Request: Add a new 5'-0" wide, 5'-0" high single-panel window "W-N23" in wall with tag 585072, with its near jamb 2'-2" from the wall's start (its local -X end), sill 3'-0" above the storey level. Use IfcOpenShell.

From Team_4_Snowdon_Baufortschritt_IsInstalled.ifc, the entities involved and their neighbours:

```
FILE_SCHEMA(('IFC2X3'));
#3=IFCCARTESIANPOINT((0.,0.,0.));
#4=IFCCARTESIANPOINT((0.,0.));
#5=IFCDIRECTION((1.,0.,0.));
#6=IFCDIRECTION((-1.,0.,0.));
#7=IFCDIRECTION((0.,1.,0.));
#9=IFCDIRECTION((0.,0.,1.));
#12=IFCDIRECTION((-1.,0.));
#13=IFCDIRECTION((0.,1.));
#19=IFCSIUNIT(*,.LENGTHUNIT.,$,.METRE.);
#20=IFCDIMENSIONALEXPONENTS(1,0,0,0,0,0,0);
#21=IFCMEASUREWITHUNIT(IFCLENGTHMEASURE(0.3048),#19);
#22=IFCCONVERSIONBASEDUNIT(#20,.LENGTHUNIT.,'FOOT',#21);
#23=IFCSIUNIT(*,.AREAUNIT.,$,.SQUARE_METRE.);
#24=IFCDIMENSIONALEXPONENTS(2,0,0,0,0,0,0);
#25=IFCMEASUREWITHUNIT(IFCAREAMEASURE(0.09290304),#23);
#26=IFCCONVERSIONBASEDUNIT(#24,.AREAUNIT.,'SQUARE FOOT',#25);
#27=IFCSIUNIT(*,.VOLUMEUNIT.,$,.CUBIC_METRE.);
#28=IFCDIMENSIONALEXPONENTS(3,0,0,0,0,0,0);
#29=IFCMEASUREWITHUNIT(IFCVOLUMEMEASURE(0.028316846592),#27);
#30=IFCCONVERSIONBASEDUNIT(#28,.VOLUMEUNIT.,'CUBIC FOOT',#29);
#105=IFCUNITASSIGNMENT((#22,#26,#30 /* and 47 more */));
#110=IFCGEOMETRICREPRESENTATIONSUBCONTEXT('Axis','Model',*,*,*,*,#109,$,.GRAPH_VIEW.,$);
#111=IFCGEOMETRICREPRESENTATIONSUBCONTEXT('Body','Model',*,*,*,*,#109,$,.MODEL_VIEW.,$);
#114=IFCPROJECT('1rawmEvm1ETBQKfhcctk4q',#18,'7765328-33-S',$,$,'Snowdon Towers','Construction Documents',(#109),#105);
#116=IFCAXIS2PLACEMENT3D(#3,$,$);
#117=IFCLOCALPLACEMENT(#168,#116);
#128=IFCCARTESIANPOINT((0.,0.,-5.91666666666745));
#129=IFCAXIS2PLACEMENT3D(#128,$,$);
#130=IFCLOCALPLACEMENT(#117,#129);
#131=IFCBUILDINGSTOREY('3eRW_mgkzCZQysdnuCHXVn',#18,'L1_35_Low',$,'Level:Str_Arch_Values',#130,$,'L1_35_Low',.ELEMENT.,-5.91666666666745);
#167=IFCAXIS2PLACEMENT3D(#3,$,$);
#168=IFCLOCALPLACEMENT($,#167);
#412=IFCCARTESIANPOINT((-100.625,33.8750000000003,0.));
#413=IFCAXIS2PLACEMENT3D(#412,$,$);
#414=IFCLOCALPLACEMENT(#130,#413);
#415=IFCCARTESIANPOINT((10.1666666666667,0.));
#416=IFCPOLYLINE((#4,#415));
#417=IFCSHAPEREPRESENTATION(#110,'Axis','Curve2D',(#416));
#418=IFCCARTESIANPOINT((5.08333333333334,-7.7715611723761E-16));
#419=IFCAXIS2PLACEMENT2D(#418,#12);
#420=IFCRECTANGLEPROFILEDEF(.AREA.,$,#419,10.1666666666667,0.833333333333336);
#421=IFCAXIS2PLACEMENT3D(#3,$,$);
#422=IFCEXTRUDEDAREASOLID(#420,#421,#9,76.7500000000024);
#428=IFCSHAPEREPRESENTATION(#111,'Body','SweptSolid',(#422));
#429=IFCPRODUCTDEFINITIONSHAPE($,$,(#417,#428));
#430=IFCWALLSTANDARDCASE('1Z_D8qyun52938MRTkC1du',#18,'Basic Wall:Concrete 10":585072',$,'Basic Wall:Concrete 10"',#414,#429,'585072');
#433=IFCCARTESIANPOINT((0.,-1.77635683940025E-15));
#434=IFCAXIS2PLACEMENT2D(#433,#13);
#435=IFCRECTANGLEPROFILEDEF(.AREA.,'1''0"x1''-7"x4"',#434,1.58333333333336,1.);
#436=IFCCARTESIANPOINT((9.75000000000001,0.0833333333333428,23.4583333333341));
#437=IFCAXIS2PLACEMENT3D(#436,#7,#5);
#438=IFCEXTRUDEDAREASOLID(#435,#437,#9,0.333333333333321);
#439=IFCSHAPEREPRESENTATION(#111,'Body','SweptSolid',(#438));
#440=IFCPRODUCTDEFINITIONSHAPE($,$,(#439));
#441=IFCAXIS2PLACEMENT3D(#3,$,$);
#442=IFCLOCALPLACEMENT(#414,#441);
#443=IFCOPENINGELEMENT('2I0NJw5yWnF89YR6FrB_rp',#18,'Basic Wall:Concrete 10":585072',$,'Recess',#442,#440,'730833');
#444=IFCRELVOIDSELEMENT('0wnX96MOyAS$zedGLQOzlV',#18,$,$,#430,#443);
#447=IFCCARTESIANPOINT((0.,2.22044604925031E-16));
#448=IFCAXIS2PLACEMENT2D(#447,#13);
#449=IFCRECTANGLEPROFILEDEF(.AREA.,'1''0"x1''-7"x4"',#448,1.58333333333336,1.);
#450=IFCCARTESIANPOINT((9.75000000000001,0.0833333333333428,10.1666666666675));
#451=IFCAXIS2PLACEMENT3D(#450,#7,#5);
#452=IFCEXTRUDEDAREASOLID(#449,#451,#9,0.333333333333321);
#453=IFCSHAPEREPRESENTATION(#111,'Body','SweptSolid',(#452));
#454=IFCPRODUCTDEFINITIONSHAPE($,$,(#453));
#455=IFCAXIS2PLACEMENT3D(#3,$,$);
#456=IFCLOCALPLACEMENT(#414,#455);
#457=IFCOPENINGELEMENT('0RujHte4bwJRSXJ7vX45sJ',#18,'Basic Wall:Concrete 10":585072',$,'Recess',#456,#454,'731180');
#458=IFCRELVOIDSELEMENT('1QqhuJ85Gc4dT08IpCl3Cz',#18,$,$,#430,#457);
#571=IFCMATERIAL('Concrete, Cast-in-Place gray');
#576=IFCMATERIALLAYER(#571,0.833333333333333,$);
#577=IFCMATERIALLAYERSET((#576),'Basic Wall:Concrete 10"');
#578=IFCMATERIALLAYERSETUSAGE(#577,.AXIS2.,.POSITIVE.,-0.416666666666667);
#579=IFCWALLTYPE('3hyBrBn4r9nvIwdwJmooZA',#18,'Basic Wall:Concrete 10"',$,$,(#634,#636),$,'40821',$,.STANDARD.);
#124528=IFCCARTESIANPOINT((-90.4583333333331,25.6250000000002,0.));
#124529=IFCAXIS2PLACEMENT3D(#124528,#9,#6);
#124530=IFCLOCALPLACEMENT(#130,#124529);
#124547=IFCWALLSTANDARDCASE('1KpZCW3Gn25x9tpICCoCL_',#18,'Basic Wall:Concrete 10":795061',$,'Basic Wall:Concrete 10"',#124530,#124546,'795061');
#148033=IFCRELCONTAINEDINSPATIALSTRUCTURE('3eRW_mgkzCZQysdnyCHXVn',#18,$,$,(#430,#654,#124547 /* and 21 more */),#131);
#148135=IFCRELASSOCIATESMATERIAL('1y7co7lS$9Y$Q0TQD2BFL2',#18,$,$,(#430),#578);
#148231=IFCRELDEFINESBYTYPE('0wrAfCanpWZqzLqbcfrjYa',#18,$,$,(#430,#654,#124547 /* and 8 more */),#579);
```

```python
import numpy as np
import ifcopenshell
import ifcopenshell.api.feature
import ifcopenshell.api.geometry
import ifcopenshell.api.root
import ifcopenshell.api.spatial
import ifcopenshell.api.type
import ifcopenshell.geom
import ifcopenshell.util.element
import ifcopenshell.util.placement
import ifcopenshell.util.representation
import ifcopenshell.util.shape
import ifcopenshell.util.unit

model = ifcopenshell.open("Team_4_Snowdon_Baufortschritt_IsInstalled.ifc")
unit_scale = ifcopenshell.util.unit.calculate_unit_scale(model)
settings = ifcopenshell.geom.settings()


def volume(element):
    """Net volume in cubic metres, openings subtracted."""
    shape = ifcopenshell.geom.create_shape(settings, element)
    return ifcopenshell.util.shape.get_volume(shape.geometry)


wall = model.by_guid("1Z_D8qyun52938MRTkC1du")
storey = ifcopenshell.util.element.get_container(wall, ifc_class="IfcBuildingStorey")
context = ifcopenshell.util.representation.get_context(model, "Model", "Body", "MODEL_VIEW")
before = volume(wall)

width, height, from_end, sill = 1.524, 1.524, 0.6604, 0.9144  # metres

# The wall runs along its own X axis, and the end named is its -X end.
wall_shape = ifcopenshell.geom.create_shape(settings, wall)
x, y, z = ifcopenshell.util.shape.get_vertices(wall_shape.geometry).T
start = x.min() + from_end
face, thickness = float(y.min()), float(y.max() - y.min())
wall_matrix = ifcopenshell.util.placement.get_local_placement(wall.ObjectPlacement)
level = ifcopenshell.util.placement.get_local_placement(storey.ObjectPlacement)[2, 3]


def in_wall(x, y):
    """Placement at x, y metres in the wall's axes, at sill height."""
    matrix = wall_matrix.copy()
    matrix[:, 3] = wall_matrix @ np.array([x / unit_scale, y / unit_scale, 0.0, 1.0])
    matrix[2, 3] = level + sill / unit_scale
    return matrix


# Opening: a box that overshoots both wall faces by 50 mm.
opening = ifcopenshell.api.root.create_entity(model, ifc_class="IfcOpeningElement")
box = ifcopenshell.api.geometry.add_wall_representation(
    model, context=context, length=width, height=height, thickness=thickness + 0.1
)
ifcopenshell.api.geometry.assign_representation(model, product=opening, representation=box)
ifcopenshell.api.geometry.edit_object_placement(model, product=opening, matrix=in_wall(start, face - 0.05), is_si=False)
ifcopenshell.api.feature.add_feature(model, feature=opening, element=wall)

window = ifcopenshell.api.root.create_entity(model, ifc_class="IfcWindow", name="W-N23")
window.OverallWidth, window.OverallHeight = width / unit_scale, height / unit_scale
body = ifcopenshell.api.geometry.add_window_representation(
    model,
    context=context,
    overall_width=window.OverallWidth,
    overall_height=window.OverallHeight,
    partition_type="SINGLE_PANEL",
)
ifcopenshell.api.geometry.assign_representation(model, product=window, representation=body)
ifcopenshell.api.spatial.assign_container(model, products=[window], relating_structure=storey)
fills = ifcopenshell.api.feature.add_filling(model, opening=opening, element=window)
fills.OwnerHistory = window.OwnerHistory  # required in IFC2X3

# IFC2X3 keeps the operation on the window style.
style = ifcopenshell.api.root.create_entity(model, ifc_class="IfcWindowStyle", name="W-N23")
style.OperationType, style.ConstructionType = "SINGLE_PANEL", "NOTDEFINED"
style.ParameterTakesPrecedence = style.Sizeable = False
ifcopenshell.api.type.assign_type(model, related_objects=[window], relating_type=style)

# Centre the window in the wall's thickness.
ifcopenshell.api.geometry.edit_object_placement(model, product=window, matrix=in_wall(start, face), is_si=False)
window_shape = ifcopenshell.geom.create_shape(settings, window)
depth = ifcopenshell.util.shape.get_vertices(window_shape.geometry)[:, 1]
offset = face + thickness / 2 - (depth.min() + depth.max()) / 2
ifcopenshell.api.geometry.edit_object_placement(model, product=window, matrix=in_wall(start, offset), is_si=False)

after = volume(wall)

print(f"wall volume {before:.3f} -> {after:.3f} m3")

model.write("Team_4_Snowdon_Baufortschritt_IsInstalled_updated.ifc")
```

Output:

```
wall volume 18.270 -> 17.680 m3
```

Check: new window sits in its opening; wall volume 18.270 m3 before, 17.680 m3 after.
